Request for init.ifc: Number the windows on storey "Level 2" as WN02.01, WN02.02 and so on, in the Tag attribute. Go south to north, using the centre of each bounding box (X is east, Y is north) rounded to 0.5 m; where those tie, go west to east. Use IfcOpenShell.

First a look at what the model holds.

```python
import ifcopenshell
import ifcopenshell.util.element
import ifcopenshell.util.placement

model = ifcopenshell.open("init.ifc")
print(model.schema)
storey = next(s for s in model.by_type("IfcBuildingStorey") if s.Name == "Level 2")
windows = [e for e in ifcopenshell.util.element.get_decomposition(storey) if e.is_a("IfcWindow")]
for e in sorted(windows, key=lambda e: e.id()):
    origin = ifcopenshell.util.placement.get_local_placement(e.ObjectPlacement)[:3, 3]
    print(e.id(), e.Tag, e.Name, origin.round(2) + 0.0, sep=" | ")
```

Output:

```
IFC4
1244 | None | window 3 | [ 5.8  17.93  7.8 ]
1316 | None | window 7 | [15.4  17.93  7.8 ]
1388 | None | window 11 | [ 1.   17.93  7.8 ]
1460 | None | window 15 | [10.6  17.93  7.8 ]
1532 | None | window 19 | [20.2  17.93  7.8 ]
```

```python
import ifcopenshell
import ifcopenshell.geom
import ifcopenshell.util.element
import ifcopenshell.util.shape

model = ifcopenshell.open("init.ifc")
settings = ifcopenshell.geom.settings()
settings.set("use-world-coords", True)


def centre(element):
    shape = ifcopenshell.geom.create_shape(settings, element)
    return ifcopenshell.util.shape.get_bbox_centroid(shape.geometry)


storey = next(s for s in model.by_type("IfcBuildingStorey") if s.Name == "Level 2")
windows = [e for e in ifcopenshell.util.element.get_decomposition(storey) if e.is_a("IfcWindow")]

# Insertion points can sit at a corner or the storey origin, so sort by the geometry (in metres).
centres = {e: centre(e) for e in windows}
windows.sort(key=lambda e: (round(centres[e][1] / 0.5), centres[e][0]))

for i, e in enumerate(windows, start=1):
    number = f"WN02.{i:02d}"
    e.Tag = number
    print(e.id(), number)

model.write("init_updated.ifc")
```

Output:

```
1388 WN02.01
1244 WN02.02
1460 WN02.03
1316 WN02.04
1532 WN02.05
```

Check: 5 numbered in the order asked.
